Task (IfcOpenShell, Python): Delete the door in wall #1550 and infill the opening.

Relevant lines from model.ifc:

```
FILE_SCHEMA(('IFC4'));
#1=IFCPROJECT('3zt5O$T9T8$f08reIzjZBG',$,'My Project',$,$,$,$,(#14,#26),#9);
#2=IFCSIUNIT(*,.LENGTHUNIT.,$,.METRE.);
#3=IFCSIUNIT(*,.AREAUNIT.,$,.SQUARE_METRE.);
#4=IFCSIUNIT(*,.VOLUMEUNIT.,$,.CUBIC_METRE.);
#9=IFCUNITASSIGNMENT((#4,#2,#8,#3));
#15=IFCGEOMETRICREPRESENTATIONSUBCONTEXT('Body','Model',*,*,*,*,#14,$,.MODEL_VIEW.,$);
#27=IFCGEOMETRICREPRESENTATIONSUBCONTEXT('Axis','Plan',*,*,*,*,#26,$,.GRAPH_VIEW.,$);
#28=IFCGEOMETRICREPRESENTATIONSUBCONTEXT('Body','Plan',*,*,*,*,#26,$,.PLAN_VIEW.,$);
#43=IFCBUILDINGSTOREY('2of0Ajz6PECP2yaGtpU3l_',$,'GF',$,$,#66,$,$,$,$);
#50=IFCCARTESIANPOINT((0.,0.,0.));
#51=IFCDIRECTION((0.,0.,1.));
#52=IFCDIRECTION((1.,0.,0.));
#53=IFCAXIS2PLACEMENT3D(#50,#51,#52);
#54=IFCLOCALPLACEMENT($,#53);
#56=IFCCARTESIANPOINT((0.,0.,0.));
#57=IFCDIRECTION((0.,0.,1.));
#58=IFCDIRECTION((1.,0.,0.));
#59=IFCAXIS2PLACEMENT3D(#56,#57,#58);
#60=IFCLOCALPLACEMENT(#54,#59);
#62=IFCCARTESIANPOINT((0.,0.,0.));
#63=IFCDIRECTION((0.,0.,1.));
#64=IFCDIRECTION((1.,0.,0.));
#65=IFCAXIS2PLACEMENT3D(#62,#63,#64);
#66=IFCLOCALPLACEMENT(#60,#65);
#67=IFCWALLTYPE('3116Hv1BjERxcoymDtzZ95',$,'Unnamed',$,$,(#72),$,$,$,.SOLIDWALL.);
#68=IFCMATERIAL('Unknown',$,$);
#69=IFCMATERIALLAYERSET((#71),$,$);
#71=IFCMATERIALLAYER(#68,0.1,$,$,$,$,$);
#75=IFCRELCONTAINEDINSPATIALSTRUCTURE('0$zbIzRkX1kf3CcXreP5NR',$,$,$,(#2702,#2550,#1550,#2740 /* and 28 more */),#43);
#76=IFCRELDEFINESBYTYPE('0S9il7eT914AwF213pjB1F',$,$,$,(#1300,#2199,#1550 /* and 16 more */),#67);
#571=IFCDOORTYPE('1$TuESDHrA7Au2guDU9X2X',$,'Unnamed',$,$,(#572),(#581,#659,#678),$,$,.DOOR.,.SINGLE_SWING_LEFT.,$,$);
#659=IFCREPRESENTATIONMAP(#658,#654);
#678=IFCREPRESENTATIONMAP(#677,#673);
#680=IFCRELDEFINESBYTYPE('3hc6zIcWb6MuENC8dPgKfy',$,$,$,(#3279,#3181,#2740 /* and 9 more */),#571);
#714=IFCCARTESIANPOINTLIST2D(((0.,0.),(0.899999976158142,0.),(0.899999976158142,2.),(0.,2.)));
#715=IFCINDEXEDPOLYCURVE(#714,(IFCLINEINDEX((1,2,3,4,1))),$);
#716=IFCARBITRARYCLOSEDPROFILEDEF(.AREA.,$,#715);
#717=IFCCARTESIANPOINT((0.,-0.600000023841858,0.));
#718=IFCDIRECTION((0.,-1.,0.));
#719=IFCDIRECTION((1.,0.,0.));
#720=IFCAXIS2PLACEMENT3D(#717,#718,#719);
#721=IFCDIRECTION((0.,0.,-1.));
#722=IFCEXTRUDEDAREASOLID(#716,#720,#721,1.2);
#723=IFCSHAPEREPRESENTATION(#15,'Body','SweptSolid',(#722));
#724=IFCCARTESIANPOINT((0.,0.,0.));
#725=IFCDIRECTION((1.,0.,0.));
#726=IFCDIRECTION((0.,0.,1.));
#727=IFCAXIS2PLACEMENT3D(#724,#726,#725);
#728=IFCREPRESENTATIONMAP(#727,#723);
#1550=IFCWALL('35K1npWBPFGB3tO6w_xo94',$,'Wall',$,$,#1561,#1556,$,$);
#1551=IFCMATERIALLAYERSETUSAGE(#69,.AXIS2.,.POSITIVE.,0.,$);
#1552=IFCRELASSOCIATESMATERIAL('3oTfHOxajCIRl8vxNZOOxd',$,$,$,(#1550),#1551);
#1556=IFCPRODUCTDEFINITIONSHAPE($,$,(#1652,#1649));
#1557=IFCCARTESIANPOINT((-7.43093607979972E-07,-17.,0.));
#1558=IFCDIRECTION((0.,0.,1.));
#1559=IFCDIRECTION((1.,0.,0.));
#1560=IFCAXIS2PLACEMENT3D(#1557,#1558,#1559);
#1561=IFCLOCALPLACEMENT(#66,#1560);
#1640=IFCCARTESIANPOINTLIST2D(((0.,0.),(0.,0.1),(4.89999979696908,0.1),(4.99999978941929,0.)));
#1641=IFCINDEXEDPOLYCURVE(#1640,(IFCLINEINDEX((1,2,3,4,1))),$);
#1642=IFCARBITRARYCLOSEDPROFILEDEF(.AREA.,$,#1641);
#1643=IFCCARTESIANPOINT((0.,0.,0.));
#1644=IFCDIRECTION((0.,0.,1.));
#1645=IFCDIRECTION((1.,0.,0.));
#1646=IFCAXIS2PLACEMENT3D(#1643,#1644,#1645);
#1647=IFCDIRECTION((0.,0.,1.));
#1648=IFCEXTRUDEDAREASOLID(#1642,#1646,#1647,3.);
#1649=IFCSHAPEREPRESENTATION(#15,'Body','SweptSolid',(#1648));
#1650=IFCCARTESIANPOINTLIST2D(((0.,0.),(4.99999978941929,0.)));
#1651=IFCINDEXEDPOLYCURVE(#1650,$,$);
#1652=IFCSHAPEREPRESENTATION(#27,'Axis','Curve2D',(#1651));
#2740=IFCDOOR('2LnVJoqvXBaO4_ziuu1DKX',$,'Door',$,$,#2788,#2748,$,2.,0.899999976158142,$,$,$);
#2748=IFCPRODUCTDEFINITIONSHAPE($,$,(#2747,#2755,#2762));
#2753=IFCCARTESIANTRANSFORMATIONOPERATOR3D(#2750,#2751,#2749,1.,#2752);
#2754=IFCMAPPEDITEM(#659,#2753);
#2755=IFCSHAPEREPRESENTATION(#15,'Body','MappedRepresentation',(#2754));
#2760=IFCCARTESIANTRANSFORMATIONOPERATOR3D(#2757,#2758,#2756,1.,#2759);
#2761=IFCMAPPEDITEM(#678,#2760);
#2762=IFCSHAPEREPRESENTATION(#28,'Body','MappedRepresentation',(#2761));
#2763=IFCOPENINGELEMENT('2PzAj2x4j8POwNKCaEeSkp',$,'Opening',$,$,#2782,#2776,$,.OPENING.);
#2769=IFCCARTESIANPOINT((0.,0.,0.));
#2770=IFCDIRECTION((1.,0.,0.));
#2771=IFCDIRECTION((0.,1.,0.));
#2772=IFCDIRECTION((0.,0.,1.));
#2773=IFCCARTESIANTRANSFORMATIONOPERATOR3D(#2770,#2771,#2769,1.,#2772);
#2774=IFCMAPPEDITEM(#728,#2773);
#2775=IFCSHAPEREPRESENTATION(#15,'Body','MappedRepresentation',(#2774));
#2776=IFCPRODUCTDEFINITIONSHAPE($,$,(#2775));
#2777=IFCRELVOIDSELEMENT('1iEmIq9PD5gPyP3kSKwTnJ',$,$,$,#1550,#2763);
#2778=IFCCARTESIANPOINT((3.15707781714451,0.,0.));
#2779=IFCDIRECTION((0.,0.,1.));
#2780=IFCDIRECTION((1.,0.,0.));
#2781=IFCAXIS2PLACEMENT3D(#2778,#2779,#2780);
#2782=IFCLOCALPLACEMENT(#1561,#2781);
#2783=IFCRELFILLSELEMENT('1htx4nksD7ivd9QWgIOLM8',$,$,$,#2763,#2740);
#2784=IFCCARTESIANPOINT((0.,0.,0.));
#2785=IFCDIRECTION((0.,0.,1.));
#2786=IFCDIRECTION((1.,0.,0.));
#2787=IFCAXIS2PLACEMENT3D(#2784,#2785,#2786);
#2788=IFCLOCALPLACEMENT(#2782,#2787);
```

```python
import ifcopenshell
import ifcopenshell.api.feature
import ifcopenshell.api.root
import ifcopenshell.geom
import ifcopenshell.util.shape

model = ifcopenshell.open("model.ifc")
settings = ifcopenshell.geom.settings()


def volume(element):
    """Net volume in cubic metres, openings subtracted."""
    shape = ifcopenshell.geom.create_shape(settings, element)
    return ifcopenshell.util.shape.get_volume(shape.geometry)


door = model.by_guid("2LnVJoqvXBaO4_ziuu1DKX")
opening = door.FillsVoids[0].RelatingOpeningElement
wall = opening.VoidsElements[0].RelatingBuildingElement
before = volume(wall)

ifcopenshell.api.root.remove_product(model, product=door)
ifcopenshell.api.feature.remove_feature(model, feature=opening)

after = volume(wall)

print(f"wall volume {before:.3f} -> {after:.3f} m3")

model.write("model_edited.ifc")
```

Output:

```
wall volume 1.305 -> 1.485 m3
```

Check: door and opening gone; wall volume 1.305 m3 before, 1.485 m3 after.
